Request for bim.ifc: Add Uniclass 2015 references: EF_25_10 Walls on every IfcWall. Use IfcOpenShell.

First a look at what the model holds.

```python
import ifcopenshell

model = ifcopenshell.open("bim.ifc")
print(model.schema)
print("classifications:", [c.Name for c in model.by_type("IfcClassification")])
for ifc_class in ("IfcDoor", "IfcRoof", "IfcStair", "IfcWall", "IfcWindow"):
    print(ifc_class, len(model.by_type(ifc_class)))
```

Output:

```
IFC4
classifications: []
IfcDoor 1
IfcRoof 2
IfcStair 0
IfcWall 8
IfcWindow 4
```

```python
import ifcopenshell
import ifcopenshell.api.classification

model = ifcopenshell.open("bim.ifc")

system = ifcopenshell.api.classification.add_classification(model, classification="Uniclass 2015")

codes = {
    "IfcWall": ("EF_25_10", "Walls"),
}
for ifc_class, (code, name) in codes.items():
    products = model.by_type(ifc_class)
    ifcopenshell.api.classification.add_reference(
        model, products=products, classification=system, identification=code, name=name
    )
    print(code, len(products))

model.write("bim_v2.ifc")
```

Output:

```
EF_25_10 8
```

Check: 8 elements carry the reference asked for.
